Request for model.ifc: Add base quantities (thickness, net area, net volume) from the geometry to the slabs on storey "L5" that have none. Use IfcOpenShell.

First a look at what the model holds.

```python
import ifcopenshell
import ifcopenshell.util.element
import ifcopenshell.util.unit

model = ifcopenshell.open("model.ifc")
print(model.schema)
for unit_type in ("LENGTHUNIT", "AREAUNIT", "VOLUMEUNIT"):
    print(unit_type, ifcopenshell.util.unit.calculate_unit_scale(model, unit_type))
storey = next(s for s in model.by_type("IfcBuildingStorey") if s.Name == "L5")
slabs = [e for e in ifcopenshell.util.element.get_decomposition(storey) if e.is_a("IfcSlab")]
for e in sorted(slabs, key=lambda e: e.id()):
    print(e.id(), e.is_a(), e.Name, list(ifcopenshell.util.element.get_psets(e, qtos_only=True)), sep=" | ")
```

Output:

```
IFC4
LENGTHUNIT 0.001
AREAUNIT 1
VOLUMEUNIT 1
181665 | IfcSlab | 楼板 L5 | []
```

```python
import ifcopenshell
import ifcopenshell.api.pset
import ifcopenshell.geom
import ifcopenshell.util.element
import ifcopenshell.util.shape
import ifcopenshell.util.unit

model = ifcopenshell.open("model.ifc")
unit_scale = ifcopenshell.util.unit.calculate_unit_scale(model)
area_scale = ifcopenshell.util.unit.calculate_unit_scale(model, "AREAUNIT")
volume_scale = ifcopenshell.util.unit.calculate_unit_scale(model, "VOLUMEUNIT")
settings = ifcopenshell.geom.settings()

storey = next(s for s in model.by_type("IfcBuildingStorey") if s.Name == "L5")
slabs = [e for e in ifcopenshell.util.element.get_decomposition(storey) if e.is_a("IfcSlab")]

for e in sorted(slabs, key=lambda e: e.id()):
    if ifcopenshell.util.element.get_psets(e, qtos_only=True, should_inherit=False):
        continue
    # Geometry comes back in metres, in the element's own axes.
    shape = ifcopenshell.geom.create_shape(settings, e)
    values = {
        "Width": ifcopenshell.util.shape.get_z(shape.geometry) / unit_scale,
        "NetArea": ifcopenshell.util.shape.get_footprint_area(shape.geometry) / area_scale,
        "NetVolume": ifcopenshell.util.shape.get_volume(shape.geometry) / volume_scale,
    }
    qto = ifcopenshell.api.pset.add_qto(model, product=e, name="Qto_SlabBaseQuantities")
    ifcopenshell.api.pset.edit_qto(model, qto=qto, properties=values)
    print(e.id(), {k: round(v, 3) for k, v in values.items()})

model.write("model_v2.ifc")
```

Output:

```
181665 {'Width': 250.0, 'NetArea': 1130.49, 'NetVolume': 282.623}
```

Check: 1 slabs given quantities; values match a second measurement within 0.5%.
